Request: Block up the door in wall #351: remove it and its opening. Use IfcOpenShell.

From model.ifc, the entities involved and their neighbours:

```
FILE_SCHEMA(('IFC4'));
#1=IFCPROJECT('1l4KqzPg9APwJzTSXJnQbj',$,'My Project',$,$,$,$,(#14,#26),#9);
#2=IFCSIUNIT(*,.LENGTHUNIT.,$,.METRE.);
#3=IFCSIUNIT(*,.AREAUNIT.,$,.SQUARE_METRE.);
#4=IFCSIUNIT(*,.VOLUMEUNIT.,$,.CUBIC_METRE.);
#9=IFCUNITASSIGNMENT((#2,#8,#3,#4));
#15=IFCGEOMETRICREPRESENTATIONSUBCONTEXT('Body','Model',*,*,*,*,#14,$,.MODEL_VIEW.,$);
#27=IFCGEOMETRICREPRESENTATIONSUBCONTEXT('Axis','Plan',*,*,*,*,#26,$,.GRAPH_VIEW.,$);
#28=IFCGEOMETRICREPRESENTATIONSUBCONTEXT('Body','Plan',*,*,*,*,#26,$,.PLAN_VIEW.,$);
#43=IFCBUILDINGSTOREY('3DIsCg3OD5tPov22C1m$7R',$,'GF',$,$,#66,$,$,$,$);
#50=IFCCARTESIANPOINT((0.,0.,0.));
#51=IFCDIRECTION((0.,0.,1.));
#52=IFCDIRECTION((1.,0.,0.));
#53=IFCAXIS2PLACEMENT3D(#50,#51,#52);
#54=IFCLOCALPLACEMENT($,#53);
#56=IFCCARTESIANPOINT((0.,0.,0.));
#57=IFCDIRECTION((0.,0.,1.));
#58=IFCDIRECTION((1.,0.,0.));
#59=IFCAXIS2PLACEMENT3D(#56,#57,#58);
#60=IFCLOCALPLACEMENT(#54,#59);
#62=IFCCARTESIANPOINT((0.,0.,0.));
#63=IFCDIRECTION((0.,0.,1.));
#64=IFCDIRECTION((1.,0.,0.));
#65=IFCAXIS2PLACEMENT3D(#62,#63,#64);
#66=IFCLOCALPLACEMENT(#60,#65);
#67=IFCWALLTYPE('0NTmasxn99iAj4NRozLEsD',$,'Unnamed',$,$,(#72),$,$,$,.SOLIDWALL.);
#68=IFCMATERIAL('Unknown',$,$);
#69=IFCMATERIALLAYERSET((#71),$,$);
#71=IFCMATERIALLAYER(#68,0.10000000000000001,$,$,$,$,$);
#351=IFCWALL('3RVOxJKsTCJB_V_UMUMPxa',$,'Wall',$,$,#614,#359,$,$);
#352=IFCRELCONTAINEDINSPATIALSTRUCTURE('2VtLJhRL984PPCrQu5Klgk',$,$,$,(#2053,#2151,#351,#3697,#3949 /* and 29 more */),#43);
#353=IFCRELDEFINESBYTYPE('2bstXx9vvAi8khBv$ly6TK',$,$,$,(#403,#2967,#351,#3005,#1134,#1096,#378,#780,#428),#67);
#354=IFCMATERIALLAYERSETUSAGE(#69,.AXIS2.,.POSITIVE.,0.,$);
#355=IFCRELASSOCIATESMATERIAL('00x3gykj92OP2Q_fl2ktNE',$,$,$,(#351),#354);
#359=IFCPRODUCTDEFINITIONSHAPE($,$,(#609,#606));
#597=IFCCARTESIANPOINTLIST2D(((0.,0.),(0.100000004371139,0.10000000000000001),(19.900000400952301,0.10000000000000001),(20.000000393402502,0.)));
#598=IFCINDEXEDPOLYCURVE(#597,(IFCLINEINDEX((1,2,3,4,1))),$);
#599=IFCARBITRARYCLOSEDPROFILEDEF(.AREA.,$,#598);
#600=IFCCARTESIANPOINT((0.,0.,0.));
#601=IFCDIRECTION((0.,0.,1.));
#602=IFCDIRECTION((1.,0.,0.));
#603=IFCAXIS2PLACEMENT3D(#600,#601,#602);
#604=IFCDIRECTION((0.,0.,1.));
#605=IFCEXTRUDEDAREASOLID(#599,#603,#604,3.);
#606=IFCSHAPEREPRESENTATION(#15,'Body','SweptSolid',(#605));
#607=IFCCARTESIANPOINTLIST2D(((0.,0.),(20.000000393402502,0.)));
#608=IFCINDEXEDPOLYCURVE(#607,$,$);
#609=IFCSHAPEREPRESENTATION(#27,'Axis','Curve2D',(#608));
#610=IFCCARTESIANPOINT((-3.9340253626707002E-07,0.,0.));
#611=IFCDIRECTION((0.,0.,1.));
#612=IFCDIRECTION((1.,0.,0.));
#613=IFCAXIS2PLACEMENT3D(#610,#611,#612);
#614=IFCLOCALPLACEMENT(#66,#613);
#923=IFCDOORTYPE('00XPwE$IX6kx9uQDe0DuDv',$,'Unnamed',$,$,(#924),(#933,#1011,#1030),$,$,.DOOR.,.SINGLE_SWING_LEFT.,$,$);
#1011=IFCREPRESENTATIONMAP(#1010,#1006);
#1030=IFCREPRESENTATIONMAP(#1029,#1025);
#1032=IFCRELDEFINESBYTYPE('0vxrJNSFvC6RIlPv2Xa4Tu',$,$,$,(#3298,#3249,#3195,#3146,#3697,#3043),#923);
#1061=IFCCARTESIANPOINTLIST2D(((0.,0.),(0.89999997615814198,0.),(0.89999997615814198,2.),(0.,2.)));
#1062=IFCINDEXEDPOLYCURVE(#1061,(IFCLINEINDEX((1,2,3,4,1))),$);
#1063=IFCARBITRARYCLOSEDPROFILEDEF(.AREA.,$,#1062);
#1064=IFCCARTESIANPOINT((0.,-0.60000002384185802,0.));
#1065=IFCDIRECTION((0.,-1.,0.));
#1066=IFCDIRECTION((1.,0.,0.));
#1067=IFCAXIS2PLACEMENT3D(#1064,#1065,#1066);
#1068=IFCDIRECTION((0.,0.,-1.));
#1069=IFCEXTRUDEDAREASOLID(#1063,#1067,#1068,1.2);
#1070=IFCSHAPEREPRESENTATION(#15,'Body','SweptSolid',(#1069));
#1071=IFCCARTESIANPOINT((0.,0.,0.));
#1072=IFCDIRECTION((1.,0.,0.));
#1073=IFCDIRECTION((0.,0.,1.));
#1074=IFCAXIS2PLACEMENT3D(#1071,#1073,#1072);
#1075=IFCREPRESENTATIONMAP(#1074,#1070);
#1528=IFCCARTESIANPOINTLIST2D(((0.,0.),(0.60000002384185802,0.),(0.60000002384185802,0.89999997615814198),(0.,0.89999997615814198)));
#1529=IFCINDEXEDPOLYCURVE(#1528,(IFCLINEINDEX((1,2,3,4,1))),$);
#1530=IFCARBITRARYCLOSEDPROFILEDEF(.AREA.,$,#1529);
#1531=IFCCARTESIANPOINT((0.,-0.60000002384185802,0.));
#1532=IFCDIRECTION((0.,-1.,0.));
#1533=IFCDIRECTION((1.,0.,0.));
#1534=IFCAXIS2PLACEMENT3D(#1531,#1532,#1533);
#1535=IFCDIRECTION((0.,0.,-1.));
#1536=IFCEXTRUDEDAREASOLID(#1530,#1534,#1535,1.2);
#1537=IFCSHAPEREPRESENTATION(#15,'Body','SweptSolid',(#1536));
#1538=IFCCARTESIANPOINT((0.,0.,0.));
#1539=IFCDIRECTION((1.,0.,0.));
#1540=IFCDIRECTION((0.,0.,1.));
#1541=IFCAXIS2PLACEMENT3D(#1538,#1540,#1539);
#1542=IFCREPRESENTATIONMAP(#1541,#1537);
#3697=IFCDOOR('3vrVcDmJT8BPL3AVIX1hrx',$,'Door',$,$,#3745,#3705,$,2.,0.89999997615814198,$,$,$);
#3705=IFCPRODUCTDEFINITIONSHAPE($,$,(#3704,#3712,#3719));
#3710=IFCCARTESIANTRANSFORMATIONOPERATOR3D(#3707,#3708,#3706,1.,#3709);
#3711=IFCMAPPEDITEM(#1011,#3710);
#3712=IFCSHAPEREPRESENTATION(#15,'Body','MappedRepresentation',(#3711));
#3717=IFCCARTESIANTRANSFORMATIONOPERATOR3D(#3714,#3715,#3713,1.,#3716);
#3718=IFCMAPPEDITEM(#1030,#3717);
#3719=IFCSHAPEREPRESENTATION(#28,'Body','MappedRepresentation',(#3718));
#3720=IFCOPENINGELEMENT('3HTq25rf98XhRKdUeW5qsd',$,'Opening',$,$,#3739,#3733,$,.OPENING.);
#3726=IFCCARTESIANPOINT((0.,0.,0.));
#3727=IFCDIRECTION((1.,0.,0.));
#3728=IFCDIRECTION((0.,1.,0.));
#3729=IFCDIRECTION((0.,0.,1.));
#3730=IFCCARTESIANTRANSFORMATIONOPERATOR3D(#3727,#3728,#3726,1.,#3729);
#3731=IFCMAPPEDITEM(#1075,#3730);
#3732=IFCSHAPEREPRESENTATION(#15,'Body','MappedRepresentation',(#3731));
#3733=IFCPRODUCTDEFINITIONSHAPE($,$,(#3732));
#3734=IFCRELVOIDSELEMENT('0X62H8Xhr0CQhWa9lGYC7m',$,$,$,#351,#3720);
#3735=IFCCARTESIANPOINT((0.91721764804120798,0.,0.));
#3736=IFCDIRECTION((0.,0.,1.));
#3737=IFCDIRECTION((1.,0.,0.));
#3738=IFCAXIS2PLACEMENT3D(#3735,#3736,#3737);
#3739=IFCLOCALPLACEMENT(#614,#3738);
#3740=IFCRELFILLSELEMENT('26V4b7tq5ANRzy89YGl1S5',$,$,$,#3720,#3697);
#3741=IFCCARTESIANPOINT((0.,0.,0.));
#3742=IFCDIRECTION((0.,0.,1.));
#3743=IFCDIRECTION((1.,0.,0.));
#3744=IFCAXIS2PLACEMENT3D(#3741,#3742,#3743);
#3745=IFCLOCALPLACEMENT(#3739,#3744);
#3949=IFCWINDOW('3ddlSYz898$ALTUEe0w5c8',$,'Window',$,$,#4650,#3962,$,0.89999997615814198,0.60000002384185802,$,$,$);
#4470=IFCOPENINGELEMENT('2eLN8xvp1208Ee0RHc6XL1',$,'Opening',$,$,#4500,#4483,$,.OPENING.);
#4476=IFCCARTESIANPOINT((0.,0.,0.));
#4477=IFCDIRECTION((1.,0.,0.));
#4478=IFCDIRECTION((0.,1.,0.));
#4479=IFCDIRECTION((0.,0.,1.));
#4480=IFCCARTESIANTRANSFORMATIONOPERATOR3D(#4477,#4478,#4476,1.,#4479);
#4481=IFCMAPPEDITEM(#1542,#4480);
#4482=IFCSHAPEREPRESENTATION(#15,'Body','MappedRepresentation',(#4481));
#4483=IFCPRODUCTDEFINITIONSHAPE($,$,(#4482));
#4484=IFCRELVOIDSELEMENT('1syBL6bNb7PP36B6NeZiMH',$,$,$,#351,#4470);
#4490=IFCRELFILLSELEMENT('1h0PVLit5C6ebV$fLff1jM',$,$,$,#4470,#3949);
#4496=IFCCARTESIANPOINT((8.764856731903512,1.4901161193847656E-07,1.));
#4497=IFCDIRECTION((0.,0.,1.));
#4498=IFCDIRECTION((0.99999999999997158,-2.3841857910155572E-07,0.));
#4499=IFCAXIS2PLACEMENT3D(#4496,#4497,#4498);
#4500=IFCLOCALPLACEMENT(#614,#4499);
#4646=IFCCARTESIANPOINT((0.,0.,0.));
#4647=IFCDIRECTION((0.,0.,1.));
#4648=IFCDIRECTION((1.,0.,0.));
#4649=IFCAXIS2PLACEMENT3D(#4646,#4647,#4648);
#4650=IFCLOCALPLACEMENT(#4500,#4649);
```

```python
import ifcopenshell
import ifcopenshell.api.feature
import ifcopenshell.api.root
import ifcopenshell.geom
import ifcopenshell.util.shape

model = ifcopenshell.open("model.ifc")
settings = ifcopenshell.geom.settings()


def volume(element):
    """Net volume in cubic metres, openings subtracted."""
    shape = ifcopenshell.geom.create_shape(settings, element)
    return ifcopenshell.util.shape.get_volume(shape.geometry)


door = model.by_guid("3vrVcDmJT8BPL3AVIX1hrx")
opening = door.FillsVoids[0].RelatingOpeningElement
wall = opening.VoidsElements[0].RelatingBuildingElement
before = volume(wall)

ifcopenshell.api.root.remove_product(model, product=door)
ifcopenshell.api.feature.remove_feature(model, feature=opening)

after = volume(wall)

print(f"wall volume {before:.3f} -> {after:.3f} m3")

model.write("model-out.ifc")
```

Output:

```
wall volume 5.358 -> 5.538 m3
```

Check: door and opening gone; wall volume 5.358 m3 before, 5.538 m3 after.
